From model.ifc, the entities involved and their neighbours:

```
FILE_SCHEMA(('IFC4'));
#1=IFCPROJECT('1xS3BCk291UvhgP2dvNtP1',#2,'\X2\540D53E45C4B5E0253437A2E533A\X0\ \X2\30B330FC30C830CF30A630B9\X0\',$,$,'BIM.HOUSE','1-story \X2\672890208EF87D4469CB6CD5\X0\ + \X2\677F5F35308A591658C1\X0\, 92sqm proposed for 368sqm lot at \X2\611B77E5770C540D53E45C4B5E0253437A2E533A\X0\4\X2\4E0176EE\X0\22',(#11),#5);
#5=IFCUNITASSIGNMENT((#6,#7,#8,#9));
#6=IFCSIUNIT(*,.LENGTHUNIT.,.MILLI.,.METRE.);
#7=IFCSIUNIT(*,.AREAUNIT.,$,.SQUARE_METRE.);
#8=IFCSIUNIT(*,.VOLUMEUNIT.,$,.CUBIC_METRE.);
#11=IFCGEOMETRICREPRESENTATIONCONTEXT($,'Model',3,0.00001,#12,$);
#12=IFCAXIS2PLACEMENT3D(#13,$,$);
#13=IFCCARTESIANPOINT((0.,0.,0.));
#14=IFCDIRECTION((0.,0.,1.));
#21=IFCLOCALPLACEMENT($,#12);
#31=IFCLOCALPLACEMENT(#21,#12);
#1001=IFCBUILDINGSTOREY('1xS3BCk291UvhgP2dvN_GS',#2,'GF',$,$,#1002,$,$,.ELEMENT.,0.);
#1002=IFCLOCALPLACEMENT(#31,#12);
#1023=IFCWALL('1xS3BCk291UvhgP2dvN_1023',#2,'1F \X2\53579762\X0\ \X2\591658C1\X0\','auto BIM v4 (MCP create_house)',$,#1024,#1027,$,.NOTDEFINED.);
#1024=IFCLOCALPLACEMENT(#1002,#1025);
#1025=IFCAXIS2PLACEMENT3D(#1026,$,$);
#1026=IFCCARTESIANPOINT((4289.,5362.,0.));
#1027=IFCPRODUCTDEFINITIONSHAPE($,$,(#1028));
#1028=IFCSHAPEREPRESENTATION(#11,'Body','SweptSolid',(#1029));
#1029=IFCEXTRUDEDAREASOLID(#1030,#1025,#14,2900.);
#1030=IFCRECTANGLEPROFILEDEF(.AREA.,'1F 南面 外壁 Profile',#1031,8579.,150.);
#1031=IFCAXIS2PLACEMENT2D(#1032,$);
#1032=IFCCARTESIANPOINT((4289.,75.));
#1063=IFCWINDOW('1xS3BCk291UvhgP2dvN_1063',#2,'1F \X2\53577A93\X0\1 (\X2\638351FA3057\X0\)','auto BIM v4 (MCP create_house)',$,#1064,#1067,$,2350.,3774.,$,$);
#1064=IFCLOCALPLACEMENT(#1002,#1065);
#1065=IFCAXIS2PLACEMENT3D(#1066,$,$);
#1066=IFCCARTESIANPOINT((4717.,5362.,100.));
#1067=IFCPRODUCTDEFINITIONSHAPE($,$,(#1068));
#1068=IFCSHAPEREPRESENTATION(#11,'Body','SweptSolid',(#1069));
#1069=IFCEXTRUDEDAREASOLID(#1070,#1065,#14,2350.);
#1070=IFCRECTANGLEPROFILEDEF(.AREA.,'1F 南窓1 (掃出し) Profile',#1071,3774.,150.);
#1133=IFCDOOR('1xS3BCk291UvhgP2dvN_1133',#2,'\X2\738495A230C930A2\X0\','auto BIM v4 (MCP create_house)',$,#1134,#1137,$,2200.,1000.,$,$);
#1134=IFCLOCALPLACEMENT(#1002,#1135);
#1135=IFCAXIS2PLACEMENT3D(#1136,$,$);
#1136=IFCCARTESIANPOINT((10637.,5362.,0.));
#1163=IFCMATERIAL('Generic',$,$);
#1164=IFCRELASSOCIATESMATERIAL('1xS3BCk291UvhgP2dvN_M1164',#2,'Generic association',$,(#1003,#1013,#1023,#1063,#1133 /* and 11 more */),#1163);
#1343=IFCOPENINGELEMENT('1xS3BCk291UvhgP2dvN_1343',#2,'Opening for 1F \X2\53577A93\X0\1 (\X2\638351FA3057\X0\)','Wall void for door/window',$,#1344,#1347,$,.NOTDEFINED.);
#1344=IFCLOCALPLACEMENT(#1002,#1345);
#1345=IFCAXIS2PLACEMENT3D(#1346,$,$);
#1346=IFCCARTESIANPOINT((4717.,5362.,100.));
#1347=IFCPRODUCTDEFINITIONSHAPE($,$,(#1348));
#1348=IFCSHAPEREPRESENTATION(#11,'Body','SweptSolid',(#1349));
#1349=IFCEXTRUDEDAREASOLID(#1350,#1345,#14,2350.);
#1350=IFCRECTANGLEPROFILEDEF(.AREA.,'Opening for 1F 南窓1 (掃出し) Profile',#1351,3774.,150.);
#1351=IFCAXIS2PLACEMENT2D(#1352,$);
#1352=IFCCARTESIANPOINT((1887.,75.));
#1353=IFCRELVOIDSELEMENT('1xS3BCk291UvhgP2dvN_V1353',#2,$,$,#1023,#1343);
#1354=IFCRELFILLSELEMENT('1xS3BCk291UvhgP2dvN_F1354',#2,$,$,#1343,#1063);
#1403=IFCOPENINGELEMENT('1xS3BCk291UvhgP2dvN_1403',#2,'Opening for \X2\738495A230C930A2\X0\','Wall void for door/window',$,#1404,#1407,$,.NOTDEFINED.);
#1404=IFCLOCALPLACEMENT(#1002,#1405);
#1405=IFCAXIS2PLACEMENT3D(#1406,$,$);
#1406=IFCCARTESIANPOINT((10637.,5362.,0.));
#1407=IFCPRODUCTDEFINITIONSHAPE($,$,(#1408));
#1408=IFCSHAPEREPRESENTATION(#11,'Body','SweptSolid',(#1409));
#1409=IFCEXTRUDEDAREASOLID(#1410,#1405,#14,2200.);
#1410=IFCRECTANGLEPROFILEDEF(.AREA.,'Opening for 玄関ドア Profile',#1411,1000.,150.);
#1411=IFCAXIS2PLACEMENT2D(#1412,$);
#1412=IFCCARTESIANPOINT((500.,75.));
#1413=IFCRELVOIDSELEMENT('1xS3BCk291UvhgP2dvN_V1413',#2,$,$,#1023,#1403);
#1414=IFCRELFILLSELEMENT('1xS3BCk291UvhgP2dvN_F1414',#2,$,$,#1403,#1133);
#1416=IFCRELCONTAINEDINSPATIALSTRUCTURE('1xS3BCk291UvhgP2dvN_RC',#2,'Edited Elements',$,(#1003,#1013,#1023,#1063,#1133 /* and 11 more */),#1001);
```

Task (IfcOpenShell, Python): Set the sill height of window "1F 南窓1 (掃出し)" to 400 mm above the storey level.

```python
import numpy as np
import ifcopenshell
import ifcopenshell.api.geometry
import ifcopenshell.geom
import ifcopenshell.util.element
import ifcopenshell.util.placement
import ifcopenshell.util.shape
import ifcopenshell.util.unit

model = ifcopenshell.open("model.ifc")
unit_scale = ifcopenshell.util.unit.calculate_unit_scale(model)

window = model.by_guid("1xS3BCk291UvhgP2dvN_1063")
opening = window.FillsVoids[0].RelatingOpeningElement
storey = ifcopenshell.util.element.get_container(window, ifc_class="IfcBuildingStorey")
level = ifcopenshell.util.placement.get_local_placement(storey.ObjectPlacement)[2, 3]

# The opening's origin need not be at the sill, so measure its lowest point.
shape = ifcopenshell.geom.create_shape(ifcopenshell.geom.settings(), opening)
bottom = ifcopenshell.util.shape.get_shape_bottom_elevation(shape, shape.geometry) / unit_scale
dz = level + 400.0 - bottom

shift = np.array([0.0, 0.0, dz])
# The window is not placed relative to its opening, so move both.
for product in (opening, window):
    matrix = ifcopenshell.util.placement.get_local_placement(product.ObjectPlacement)
    matrix[:3, 3] += shift
    ifcopenshell.api.geometry.edit_object_placement(model, product=product, matrix=matrix, is_si=False)

print(f"moved by {dz * unit_scale:+.3f} m")

model.write("model_updated.ifc")
```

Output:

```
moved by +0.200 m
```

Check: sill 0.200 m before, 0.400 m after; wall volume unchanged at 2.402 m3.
